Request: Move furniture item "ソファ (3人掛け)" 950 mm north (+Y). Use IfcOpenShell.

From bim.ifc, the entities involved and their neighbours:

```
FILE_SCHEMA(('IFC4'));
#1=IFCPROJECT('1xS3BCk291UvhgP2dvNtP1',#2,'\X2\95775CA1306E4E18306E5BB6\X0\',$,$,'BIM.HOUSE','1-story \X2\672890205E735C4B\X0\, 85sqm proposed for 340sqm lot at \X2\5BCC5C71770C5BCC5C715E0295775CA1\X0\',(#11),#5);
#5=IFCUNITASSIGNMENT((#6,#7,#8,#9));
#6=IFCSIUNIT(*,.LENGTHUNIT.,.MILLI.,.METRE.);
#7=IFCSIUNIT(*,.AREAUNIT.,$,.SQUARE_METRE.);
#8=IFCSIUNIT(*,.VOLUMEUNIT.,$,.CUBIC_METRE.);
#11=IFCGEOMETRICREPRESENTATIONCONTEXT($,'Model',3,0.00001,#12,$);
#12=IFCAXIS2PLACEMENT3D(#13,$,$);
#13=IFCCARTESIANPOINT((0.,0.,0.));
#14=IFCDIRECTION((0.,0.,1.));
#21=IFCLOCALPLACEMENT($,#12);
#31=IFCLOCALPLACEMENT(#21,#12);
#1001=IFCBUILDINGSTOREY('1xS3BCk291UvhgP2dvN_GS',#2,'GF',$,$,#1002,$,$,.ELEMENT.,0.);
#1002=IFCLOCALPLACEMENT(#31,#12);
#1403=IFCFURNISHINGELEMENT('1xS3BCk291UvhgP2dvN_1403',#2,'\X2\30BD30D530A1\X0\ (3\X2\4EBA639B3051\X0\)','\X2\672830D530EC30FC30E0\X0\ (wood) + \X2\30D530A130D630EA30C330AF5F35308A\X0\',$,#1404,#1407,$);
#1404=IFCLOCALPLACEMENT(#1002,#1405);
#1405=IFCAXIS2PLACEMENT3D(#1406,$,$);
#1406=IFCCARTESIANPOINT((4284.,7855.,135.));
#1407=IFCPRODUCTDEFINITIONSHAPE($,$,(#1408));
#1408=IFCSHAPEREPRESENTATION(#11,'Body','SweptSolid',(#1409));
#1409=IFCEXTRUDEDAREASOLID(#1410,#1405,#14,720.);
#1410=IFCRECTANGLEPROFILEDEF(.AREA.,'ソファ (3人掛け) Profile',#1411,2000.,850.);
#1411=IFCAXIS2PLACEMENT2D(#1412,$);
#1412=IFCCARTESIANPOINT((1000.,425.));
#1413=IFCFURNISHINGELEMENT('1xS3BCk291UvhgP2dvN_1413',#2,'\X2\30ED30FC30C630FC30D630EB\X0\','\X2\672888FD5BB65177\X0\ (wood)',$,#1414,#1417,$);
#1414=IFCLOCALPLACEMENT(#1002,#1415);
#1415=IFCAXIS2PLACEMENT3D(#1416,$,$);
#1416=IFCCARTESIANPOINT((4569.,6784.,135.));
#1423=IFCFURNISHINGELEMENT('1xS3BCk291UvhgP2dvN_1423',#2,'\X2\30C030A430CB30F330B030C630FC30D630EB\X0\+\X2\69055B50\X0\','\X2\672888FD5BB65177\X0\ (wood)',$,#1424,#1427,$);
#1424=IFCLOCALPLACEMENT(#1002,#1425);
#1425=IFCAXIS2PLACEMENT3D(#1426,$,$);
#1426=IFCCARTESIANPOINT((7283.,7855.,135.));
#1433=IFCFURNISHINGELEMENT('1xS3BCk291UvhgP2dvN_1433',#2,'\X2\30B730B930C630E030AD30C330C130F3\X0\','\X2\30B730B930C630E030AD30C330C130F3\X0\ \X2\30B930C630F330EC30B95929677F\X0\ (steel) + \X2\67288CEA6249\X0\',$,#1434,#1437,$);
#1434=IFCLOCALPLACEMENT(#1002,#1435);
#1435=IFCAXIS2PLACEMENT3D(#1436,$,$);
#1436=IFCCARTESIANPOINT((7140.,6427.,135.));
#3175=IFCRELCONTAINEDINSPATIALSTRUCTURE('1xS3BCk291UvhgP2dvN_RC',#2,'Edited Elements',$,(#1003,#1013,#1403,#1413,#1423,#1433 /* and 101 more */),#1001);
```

```python
import ifcopenshell
import ifcopenshell.api.geometry
import ifcopenshell.util.placement
import ifcopenshell.util.unit

model = ifcopenshell.open("bim.ifc")
unit_scale = ifcopenshell.util.unit.calculate_unit_scale(model)

item = model.by_guid("1xS3BCk291UvhgP2dvN_1403")
matrix = ifcopenshell.util.placement.get_local_placement(item.ObjectPlacement)
matrix[1, 3] += 0.95 / unit_scale
ifcopenshell.api.geometry.edit_object_placement(model, product=item, matrix=matrix, is_si=False)

print(ifcopenshell.util.placement.get_local_placement(item.ObjectPlacement).round(3) + 0.0)

model.write("bim_updated.ifc")
```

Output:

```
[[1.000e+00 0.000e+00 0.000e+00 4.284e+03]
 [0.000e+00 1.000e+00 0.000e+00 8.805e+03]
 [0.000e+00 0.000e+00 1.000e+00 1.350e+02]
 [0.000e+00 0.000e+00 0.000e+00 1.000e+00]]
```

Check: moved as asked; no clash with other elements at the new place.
